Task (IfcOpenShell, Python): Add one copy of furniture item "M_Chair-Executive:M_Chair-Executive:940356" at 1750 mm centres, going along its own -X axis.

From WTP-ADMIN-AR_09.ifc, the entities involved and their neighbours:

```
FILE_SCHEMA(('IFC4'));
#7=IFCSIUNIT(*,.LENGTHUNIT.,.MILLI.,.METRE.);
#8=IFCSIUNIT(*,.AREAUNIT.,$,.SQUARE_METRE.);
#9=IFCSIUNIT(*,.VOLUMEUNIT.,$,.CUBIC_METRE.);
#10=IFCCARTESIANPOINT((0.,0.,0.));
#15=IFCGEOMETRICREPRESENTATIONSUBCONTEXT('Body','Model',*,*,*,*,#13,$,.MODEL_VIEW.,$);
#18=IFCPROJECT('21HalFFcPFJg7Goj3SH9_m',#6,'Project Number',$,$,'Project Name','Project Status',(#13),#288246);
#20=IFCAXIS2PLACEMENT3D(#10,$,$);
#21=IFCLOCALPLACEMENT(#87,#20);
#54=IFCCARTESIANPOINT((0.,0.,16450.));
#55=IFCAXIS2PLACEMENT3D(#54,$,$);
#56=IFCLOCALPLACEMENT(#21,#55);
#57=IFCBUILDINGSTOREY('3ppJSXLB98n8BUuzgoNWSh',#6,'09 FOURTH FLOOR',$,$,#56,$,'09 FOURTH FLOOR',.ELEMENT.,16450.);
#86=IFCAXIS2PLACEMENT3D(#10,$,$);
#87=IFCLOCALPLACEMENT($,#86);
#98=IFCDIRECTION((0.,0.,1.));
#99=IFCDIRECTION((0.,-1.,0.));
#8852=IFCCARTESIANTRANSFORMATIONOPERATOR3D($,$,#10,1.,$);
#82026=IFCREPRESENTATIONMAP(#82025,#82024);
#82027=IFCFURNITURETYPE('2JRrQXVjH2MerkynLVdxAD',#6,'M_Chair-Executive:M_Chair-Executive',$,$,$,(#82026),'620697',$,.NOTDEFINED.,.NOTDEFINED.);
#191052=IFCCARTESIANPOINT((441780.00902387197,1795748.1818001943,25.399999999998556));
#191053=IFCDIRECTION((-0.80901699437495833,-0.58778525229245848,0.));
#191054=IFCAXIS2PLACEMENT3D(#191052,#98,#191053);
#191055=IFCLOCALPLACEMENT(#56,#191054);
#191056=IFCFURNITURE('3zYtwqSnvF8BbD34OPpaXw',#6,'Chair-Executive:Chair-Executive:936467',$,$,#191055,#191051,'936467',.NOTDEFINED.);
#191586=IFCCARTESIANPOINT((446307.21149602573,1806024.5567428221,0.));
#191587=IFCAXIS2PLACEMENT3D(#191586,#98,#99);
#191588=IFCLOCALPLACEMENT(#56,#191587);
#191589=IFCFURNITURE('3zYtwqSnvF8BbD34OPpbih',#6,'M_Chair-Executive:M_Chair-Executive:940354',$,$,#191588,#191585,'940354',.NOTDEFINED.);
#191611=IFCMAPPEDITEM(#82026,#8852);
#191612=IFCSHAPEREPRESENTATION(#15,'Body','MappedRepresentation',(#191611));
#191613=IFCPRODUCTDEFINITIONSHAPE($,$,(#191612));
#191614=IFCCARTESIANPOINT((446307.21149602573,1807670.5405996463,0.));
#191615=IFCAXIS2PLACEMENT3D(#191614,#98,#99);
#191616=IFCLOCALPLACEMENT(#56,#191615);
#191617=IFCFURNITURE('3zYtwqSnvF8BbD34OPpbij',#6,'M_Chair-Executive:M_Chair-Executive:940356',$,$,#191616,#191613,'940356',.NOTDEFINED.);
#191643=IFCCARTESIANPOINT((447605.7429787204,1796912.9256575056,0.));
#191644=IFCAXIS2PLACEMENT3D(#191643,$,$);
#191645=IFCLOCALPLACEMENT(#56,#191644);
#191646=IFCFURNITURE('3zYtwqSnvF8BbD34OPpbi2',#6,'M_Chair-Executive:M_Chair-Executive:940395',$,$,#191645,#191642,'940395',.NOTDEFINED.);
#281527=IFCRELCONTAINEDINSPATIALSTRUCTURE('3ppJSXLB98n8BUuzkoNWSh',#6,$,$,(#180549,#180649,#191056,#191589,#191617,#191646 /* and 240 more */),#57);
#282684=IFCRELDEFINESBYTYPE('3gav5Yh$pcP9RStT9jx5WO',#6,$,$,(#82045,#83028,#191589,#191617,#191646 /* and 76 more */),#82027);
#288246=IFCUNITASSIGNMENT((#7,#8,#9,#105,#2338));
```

```python
import ifcopenshell
import ifcopenshell.api.geometry
import ifcopenshell.api.root
import ifcopenshell.util.element
import ifcopenshell.util.placement

model = ifcopenshell.open("WTP-ADMIN-AR_09.ifc")


def reuse_history(source, copy):
    """copy_class also copies each property set's owner history, people and application; keep the originals."""
    for rel in copy.IsDefinedBy:
        if rel.is_a("IfcRelDefinesByProperties") and (history := rel.RelatingPropertyDefinition.OwnerHistory):
            rel.RelatingPropertyDefinition.OwnerHistory = source.OwnerHistory
            ifcopenshell.util.element.remove_deep2(model, history)


source = model.by_guid("3zYtwqSnvF8BbD34OPpbij")
base = ifcopenshell.util.placement.get_local_placement(source.ObjectPlacement)
step = -base[:3, 0] * 1750.0

for i in range(1, 2):
    copy = ifcopenshell.api.root.copy_class(model, product=source)
    copy.Representation = ifcopenshell.util.element.copy_deep(
        model, source.Representation, exclude=["IfcGeometricRepresentationContext", "IfcRepresentationMap"]
    )
    copy.Name = "M_Chair-Executive:M_Chair-Executive"
    copy.Tag = None
    reuse_history(source, copy)
    matrix = base.copy()
    matrix[:3, 3] += i * step
    print("added at", matrix[:3, 3].round(3) + 0.0)
    ifcopenshell.api.geometry.edit_object_placement(model, product=copy, matrix=matrix, is_si=False)

model.write("WTP-ADMIN-AR_09_v2.ifc")
```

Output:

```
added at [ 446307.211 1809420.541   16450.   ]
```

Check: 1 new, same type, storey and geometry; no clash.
